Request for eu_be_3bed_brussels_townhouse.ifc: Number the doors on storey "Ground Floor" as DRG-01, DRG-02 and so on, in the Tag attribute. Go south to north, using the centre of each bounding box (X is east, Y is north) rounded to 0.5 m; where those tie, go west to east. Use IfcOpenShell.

First a look at what the model holds.

```python
import ifcopenshell
import ifcopenshell.util.element
import ifcopenshell.util.placement

model = ifcopenshell.open("eu_be_3bed_brussels_townhouse.ifc")
print(model.schema)
storey = next(s for s in model.by_type("IfcBuildingStorey") if s.Name == "Ground Floor")
doors = [e for e in ifcopenshell.util.element.get_decomposition(storey) if e.is_a("IfcDoor")]
for e in sorted(doors, key=lambda e: e.id()):
    origin = ifcopenshell.util.placement.get_local_placement(e.ObjectPlacement)[:3, 3]
    print(e.id(), e.Tag, e.Name, origin.round(2) + 0.0, sep=" | ")
```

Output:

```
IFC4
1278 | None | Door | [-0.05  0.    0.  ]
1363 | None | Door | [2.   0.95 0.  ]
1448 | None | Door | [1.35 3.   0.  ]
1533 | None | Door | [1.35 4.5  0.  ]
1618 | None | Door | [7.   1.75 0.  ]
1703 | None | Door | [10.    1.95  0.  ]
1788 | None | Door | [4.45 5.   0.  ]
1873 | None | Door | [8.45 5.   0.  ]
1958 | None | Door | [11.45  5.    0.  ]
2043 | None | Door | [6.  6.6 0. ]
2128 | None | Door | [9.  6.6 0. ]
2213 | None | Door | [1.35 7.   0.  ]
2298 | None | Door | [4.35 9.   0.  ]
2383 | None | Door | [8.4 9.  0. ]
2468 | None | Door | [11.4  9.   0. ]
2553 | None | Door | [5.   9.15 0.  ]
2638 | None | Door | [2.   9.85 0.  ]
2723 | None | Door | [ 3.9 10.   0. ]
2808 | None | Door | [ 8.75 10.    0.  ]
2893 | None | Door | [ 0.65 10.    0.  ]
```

```python
import ifcopenshell
import ifcopenshell.geom
import ifcopenshell.util.element
import ifcopenshell.util.shape

model = ifcopenshell.open("eu_be_3bed_brussels_townhouse.ifc")
settings = ifcopenshell.geom.settings()
settings.set("use-world-coords", True)


def centre(element):
    shape = ifcopenshell.geom.create_shape(settings, element)
    return ifcopenshell.util.shape.get_bbox_centroid(shape.geometry)


storey = next(s for s in model.by_type("IfcBuildingStorey") if s.Name == "Ground Floor")
doors = [e for e in ifcopenshell.util.element.get_decomposition(storey) if e.is_a("IfcDoor")]

# Insertion points can sit at a corner or the storey origin, so sort by the geometry (in metres).
centres = {e: centre(e) for e in doors}
doors.sort(key=lambda e: (round(centres[e][1] / 0.5), centres[e][0]))

for i, e in enumerate(doors, start=1):
    number = f"DRG-{i:02d}"
    e.Tag = number
    print(e.id(), number)

model.write("eu_be_3bed_brussels_townhouse_v2.ifc")
```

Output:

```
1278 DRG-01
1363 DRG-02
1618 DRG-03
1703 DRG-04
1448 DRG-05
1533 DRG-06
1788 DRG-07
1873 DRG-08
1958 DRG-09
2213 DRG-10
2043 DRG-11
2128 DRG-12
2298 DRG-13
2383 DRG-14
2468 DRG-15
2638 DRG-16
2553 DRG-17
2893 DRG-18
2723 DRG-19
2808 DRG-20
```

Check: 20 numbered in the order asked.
